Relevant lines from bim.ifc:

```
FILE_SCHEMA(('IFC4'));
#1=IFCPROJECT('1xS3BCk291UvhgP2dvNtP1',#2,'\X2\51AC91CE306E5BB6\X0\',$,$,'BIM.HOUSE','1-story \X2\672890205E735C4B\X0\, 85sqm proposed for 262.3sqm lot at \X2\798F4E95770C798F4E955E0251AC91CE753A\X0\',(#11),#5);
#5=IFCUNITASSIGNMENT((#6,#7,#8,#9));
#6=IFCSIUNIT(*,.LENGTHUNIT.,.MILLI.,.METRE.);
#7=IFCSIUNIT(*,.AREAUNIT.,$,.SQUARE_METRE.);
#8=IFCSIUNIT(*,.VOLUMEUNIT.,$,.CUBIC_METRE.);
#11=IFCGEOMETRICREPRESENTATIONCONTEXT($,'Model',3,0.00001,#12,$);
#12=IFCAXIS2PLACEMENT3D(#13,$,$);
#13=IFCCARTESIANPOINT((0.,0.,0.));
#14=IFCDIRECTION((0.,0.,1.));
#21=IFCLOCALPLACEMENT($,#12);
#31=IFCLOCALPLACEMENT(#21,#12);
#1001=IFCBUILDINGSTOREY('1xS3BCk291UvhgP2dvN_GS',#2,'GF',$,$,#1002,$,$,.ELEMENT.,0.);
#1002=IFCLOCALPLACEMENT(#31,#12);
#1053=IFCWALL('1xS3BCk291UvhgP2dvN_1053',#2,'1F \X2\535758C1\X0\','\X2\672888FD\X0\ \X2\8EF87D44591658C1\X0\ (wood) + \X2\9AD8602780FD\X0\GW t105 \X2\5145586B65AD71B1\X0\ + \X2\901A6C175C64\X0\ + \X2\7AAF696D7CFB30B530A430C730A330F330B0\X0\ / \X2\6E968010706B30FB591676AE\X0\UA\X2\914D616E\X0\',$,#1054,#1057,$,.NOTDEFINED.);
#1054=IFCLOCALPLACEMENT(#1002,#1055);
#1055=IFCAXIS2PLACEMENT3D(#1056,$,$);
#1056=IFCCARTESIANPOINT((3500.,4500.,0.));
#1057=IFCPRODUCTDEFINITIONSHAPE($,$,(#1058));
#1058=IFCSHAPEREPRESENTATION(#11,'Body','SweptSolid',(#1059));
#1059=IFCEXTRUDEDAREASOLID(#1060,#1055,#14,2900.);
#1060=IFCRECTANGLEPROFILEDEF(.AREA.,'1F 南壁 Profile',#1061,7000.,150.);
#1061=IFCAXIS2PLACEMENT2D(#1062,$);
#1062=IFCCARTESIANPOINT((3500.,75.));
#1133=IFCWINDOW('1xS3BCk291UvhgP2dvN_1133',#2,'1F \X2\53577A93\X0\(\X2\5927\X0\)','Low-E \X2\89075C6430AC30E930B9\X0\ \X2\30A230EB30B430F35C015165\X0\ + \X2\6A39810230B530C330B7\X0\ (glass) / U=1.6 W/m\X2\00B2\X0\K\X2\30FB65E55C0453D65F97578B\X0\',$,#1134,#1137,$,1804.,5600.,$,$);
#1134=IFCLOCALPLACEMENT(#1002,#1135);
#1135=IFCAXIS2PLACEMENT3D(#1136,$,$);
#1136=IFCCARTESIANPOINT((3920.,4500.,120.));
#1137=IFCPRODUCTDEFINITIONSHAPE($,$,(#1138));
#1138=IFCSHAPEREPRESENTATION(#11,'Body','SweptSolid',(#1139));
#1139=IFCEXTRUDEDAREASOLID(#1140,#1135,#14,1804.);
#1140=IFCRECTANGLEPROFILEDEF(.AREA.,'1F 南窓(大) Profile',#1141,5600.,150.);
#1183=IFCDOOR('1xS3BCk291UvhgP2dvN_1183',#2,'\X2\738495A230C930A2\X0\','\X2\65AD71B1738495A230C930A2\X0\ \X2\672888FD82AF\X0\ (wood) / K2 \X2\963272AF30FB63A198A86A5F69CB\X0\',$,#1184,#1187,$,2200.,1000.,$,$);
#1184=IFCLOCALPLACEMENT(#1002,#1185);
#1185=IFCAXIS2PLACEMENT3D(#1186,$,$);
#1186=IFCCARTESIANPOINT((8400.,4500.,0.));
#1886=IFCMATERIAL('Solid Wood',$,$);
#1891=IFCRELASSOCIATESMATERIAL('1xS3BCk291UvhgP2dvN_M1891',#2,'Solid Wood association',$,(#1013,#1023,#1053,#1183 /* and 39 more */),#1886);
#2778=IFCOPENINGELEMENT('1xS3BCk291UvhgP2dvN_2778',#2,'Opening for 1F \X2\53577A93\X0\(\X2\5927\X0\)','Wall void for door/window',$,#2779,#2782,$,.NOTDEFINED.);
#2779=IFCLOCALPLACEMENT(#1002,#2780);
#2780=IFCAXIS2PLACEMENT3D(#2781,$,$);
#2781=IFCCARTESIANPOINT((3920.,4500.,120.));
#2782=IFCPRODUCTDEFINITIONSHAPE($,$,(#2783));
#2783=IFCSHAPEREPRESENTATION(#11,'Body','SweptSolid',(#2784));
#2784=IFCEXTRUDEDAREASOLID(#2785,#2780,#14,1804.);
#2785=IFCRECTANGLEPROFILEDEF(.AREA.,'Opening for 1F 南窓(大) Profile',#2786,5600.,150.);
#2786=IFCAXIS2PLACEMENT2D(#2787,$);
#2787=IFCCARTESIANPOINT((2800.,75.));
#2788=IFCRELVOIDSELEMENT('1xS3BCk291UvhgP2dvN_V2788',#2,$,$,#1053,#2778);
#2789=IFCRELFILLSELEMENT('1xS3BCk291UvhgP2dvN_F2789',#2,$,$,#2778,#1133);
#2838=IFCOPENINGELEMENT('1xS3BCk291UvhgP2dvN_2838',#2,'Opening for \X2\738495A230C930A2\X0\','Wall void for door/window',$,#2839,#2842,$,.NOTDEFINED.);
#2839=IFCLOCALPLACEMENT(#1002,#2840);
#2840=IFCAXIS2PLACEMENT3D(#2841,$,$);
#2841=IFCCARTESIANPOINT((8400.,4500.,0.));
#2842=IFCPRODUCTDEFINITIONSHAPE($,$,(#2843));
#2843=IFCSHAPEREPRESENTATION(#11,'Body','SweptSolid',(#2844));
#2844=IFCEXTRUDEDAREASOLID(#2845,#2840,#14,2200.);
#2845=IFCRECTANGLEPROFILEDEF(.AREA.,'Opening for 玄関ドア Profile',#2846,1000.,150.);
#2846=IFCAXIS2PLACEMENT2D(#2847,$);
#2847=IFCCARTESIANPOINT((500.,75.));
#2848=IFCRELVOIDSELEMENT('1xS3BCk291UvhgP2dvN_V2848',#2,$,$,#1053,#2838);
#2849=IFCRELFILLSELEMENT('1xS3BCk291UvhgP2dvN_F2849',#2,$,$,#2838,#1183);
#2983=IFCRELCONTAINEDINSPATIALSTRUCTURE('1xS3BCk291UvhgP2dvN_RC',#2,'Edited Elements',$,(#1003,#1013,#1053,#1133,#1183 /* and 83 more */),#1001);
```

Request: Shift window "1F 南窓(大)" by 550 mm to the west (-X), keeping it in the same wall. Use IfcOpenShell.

```python
import ifcopenshell
import ifcopenshell.api.geometry
import ifcopenshell.util.placement

model = ifcopenshell.open("bim.ifc")

window = model.by_id(1133)
opening = window.FillsVoids[0].RelatingOpeningElement
wall = opening.VoidsElements[0].RelatingBuildingElement

wall_matrix = ifcopenshell.util.placement.get_local_placement(wall.ObjectPlacement)
shift = wall_matrix[:3, 0] * -550.0
before = ifcopenshell.util.placement.get_local_placement(window.ObjectPlacement)[:3, 3].copy()

# The window is not placed relative to its opening, so move both.
for product in (opening, window):
    matrix = ifcopenshell.util.placement.get_local_placement(product.ObjectPlacement)
    matrix[:3, 3] += shift
    ifcopenshell.api.geometry.edit_object_placement(model, product=product, matrix=matrix, is_si=False)

after = ifcopenshell.util.placement.get_local_placement(window.ObjectPlacement)[:3, 3]
print("window moved by", (after - before).round(3) + 0.0)

model.write("bim_updated.ifc")
```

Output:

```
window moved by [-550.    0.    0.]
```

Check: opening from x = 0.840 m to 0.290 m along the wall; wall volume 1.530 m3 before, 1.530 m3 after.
